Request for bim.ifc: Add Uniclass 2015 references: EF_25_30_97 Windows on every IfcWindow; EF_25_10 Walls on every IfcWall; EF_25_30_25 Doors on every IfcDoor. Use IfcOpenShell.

First a look at what the model holds.

```python
import ifcopenshell

model = ifcopenshell.open("bim.ifc")
print(model.schema)
print("classifications:", [c.Name for c in model.by_type("IfcClassification")])
for ifc_class in ("IfcDoor", "IfcRoof", "IfcStair", "IfcWall", "IfcWindow"):
    print(ifc_class, len(model.by_type(ifc_class)))
```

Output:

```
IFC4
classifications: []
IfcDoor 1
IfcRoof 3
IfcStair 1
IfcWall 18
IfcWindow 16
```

```python
import ifcopenshell
import ifcopenshell.api.classification

model = ifcopenshell.open("bim.ifc")

system = ifcopenshell.api.classification.add_classification(model, classification="Uniclass 2015")

codes = {
    "IfcWindow": ("EF_25_30_97", "Windows"),
    "IfcWall": ("EF_25_10", "Walls"),
    "IfcDoor": ("EF_25_30_25", "Doors"),
}
for ifc_class, (code, name) in codes.items():
    products = model.by_type(ifc_class)
    ifcopenshell.api.classification.add_reference(
        model, products=products, classification=system, identification=code, name=name
    )
    print(code, len(products))

model.write("bim_rev.ifc")
```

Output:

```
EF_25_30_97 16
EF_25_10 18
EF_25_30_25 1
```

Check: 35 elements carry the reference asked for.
